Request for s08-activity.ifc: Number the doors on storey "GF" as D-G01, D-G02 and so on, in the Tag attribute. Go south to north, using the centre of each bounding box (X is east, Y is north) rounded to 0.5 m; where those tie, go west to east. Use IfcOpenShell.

First a look at what the model holds.

```python
import ifcopenshell
import ifcopenshell.util.element
import ifcopenshell.util.placement

model = ifcopenshell.open("s08-activity.ifc")
print(model.schema)
storey = next(s for s in model.by_type("IfcBuildingStorey") if s.Name == "GF")
doors = [e for e in ifcopenshell.util.element.get_decomposition(storey) if e.is_a("IfcDoor")]
for e in sorted(doors, key=lambda e: e.id()):
    origin = ifcopenshell.util.placement.get_local_placement(e.ObjectPlacement)[:3, 3]
    print(e.id(), e.Tag, e.Name, origin.round(2) + 0.0, sep=" | ")
```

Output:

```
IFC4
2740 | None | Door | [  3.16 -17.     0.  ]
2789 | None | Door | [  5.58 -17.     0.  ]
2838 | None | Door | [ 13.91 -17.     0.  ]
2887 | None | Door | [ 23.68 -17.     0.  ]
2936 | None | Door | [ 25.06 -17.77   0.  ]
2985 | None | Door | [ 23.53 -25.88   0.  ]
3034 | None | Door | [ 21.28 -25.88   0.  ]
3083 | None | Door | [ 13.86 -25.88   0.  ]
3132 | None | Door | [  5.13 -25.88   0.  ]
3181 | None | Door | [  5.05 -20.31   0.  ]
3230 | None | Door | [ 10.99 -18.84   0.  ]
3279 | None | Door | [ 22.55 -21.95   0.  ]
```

```python
import ifcopenshell
import ifcopenshell.geom
import ifcopenshell.util.element
import ifcopenshell.util.shape

model = ifcopenshell.open("s08-activity.ifc")
settings = ifcopenshell.geom.settings()
settings.set("use-world-coords", True)


def centre(element):
    shape = ifcopenshell.geom.create_shape(settings, element)
    return ifcopenshell.util.shape.get_bbox_centroid(shape.geometry)


storey = next(s for s in model.by_type("IfcBuildingStorey") if s.Name == "GF")
doors = [e for e in ifcopenshell.util.element.get_decomposition(storey) if e.is_a("IfcDoor")]

# Insertion points can sit at a corner or the storey origin, so sort by the geometry (in metres).
centres = {e: centre(e) for e in doors}
doors.sort(key=lambda e: (round(centres[e][1] / 0.5), centres[e][0]))

for i, e in enumerate(doors, start=1):
    number = f"D-G{i:02d}"
    e.Tag = number
    print(e.id(), number)

model.write("s08-activity-out.ifc")
```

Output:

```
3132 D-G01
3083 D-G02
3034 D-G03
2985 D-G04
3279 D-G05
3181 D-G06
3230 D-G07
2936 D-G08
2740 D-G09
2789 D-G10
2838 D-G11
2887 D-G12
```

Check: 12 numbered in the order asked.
